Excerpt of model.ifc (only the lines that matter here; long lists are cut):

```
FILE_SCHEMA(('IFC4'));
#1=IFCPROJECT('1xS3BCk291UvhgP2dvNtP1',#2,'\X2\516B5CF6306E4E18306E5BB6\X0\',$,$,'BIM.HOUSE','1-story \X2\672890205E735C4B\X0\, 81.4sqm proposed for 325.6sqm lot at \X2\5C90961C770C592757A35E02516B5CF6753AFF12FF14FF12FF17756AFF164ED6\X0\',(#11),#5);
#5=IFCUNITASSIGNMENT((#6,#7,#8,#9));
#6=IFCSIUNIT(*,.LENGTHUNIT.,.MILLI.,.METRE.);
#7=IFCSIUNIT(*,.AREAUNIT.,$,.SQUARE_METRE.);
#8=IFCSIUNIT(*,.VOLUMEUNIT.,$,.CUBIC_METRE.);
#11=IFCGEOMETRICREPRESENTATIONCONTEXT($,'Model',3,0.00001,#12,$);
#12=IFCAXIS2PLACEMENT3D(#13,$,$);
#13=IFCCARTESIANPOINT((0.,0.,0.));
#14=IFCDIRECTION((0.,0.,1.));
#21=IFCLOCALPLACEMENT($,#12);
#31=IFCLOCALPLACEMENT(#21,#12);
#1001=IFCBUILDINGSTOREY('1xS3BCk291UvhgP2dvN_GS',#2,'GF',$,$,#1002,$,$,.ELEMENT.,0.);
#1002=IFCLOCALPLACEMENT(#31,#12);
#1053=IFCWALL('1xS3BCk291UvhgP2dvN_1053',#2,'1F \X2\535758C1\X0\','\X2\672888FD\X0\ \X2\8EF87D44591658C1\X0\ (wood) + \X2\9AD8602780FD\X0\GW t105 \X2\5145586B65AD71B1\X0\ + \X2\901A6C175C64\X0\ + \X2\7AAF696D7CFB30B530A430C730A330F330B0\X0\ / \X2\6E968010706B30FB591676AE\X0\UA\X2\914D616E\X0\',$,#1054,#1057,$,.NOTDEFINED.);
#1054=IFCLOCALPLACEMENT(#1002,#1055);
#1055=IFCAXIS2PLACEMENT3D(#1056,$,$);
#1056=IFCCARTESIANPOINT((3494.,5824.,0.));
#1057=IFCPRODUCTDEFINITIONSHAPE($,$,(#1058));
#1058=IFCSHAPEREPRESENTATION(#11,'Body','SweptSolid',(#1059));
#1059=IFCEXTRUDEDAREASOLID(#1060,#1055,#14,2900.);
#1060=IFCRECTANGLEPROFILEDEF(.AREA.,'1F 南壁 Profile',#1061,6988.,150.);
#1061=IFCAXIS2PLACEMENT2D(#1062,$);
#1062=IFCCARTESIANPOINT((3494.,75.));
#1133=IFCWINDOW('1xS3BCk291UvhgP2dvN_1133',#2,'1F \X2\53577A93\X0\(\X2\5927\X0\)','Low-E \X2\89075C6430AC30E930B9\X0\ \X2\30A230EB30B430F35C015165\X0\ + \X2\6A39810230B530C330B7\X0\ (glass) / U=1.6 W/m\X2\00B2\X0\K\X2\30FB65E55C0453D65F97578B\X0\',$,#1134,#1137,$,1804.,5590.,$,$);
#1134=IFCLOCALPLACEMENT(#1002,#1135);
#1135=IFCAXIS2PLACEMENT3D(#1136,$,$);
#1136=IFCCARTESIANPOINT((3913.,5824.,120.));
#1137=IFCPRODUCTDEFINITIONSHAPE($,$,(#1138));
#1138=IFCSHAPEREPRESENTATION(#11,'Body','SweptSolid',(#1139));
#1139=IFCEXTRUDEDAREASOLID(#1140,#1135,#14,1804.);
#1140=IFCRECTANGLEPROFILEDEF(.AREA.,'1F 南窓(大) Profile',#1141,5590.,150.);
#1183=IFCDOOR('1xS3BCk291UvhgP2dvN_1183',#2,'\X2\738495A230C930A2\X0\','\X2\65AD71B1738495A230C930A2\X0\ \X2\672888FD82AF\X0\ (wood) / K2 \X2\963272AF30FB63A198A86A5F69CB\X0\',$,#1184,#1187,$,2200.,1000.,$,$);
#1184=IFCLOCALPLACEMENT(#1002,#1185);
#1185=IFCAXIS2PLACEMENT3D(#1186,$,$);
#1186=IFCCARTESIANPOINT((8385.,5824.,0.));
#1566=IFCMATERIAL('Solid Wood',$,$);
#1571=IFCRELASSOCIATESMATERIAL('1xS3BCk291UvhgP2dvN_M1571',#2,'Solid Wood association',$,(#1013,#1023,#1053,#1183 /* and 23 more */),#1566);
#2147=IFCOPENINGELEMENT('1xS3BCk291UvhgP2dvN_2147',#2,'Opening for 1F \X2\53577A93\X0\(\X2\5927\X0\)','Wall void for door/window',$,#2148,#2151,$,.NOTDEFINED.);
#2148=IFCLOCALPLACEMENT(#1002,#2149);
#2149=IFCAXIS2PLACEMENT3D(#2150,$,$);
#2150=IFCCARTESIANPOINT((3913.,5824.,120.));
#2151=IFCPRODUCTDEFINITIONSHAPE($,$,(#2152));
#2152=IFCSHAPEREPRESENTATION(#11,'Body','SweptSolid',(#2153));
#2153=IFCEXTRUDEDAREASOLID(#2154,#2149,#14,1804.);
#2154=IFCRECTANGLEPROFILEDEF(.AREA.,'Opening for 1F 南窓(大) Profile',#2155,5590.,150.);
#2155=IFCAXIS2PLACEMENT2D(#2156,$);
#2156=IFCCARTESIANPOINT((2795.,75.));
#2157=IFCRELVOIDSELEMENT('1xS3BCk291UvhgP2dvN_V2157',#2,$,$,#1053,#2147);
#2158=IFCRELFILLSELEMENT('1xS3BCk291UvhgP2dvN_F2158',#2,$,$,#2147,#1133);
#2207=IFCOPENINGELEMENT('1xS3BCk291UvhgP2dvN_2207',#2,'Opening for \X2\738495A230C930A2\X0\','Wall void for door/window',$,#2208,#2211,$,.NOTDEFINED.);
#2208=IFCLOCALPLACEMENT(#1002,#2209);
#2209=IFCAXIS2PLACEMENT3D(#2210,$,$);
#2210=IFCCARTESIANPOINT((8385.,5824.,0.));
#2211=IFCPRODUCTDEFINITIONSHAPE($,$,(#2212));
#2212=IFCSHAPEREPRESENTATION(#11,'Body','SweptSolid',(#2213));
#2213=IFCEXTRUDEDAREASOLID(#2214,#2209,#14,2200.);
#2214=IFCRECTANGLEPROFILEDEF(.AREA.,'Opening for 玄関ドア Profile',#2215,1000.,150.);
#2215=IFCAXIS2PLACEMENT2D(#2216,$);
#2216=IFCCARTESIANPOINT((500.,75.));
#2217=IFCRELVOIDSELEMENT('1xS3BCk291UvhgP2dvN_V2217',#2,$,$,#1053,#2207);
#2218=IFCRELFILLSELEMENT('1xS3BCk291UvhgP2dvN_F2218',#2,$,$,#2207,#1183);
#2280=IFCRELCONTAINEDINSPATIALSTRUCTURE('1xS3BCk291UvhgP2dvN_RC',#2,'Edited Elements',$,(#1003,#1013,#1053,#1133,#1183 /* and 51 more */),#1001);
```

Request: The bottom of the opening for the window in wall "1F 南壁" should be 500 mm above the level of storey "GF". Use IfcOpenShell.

```python
import numpy as np
import ifcopenshell
import ifcopenshell.api.geometry
import ifcopenshell.geom
import ifcopenshell.util.element
import ifcopenshell.util.placement
import ifcopenshell.util.shape
import ifcopenshell.util.unit

model = ifcopenshell.open("model.ifc")
unit_scale = ifcopenshell.util.unit.calculate_unit_scale(model)

window = model.by_guid("1xS3BCk291UvhgP2dvN_1133")
opening = window.FillsVoids[0].RelatingOpeningElement
storey = ifcopenshell.util.element.get_container(window, ifc_class="IfcBuildingStorey")
level = ifcopenshell.util.placement.get_local_placement(storey.ObjectPlacement)[2, 3]

# The opening's origin need not be at the sill, so measure its lowest point.
shape = ifcopenshell.geom.create_shape(ifcopenshell.geom.settings(), opening)
bottom = ifcopenshell.util.shape.get_shape_bottom_elevation(shape, shape.geometry) / unit_scale
dz = level + 500.0 - bottom

shift = np.array([0.0, 0.0, dz])
# The window is not placed relative to its opening, so move both.
for product in (opening, window):
    matrix = ifcopenshell.util.placement.get_local_placement(product.ObjectPlacement)
    matrix[:3, 3] += shift
    ifcopenshell.api.geometry.edit_object_placement(model, product=product, matrix=matrix, is_si=False)

print(f"moved by {dz * unit_scale:+.3f} m")

model.write("model_updated.ifc")
```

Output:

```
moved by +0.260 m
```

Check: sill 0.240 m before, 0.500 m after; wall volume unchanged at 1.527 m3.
